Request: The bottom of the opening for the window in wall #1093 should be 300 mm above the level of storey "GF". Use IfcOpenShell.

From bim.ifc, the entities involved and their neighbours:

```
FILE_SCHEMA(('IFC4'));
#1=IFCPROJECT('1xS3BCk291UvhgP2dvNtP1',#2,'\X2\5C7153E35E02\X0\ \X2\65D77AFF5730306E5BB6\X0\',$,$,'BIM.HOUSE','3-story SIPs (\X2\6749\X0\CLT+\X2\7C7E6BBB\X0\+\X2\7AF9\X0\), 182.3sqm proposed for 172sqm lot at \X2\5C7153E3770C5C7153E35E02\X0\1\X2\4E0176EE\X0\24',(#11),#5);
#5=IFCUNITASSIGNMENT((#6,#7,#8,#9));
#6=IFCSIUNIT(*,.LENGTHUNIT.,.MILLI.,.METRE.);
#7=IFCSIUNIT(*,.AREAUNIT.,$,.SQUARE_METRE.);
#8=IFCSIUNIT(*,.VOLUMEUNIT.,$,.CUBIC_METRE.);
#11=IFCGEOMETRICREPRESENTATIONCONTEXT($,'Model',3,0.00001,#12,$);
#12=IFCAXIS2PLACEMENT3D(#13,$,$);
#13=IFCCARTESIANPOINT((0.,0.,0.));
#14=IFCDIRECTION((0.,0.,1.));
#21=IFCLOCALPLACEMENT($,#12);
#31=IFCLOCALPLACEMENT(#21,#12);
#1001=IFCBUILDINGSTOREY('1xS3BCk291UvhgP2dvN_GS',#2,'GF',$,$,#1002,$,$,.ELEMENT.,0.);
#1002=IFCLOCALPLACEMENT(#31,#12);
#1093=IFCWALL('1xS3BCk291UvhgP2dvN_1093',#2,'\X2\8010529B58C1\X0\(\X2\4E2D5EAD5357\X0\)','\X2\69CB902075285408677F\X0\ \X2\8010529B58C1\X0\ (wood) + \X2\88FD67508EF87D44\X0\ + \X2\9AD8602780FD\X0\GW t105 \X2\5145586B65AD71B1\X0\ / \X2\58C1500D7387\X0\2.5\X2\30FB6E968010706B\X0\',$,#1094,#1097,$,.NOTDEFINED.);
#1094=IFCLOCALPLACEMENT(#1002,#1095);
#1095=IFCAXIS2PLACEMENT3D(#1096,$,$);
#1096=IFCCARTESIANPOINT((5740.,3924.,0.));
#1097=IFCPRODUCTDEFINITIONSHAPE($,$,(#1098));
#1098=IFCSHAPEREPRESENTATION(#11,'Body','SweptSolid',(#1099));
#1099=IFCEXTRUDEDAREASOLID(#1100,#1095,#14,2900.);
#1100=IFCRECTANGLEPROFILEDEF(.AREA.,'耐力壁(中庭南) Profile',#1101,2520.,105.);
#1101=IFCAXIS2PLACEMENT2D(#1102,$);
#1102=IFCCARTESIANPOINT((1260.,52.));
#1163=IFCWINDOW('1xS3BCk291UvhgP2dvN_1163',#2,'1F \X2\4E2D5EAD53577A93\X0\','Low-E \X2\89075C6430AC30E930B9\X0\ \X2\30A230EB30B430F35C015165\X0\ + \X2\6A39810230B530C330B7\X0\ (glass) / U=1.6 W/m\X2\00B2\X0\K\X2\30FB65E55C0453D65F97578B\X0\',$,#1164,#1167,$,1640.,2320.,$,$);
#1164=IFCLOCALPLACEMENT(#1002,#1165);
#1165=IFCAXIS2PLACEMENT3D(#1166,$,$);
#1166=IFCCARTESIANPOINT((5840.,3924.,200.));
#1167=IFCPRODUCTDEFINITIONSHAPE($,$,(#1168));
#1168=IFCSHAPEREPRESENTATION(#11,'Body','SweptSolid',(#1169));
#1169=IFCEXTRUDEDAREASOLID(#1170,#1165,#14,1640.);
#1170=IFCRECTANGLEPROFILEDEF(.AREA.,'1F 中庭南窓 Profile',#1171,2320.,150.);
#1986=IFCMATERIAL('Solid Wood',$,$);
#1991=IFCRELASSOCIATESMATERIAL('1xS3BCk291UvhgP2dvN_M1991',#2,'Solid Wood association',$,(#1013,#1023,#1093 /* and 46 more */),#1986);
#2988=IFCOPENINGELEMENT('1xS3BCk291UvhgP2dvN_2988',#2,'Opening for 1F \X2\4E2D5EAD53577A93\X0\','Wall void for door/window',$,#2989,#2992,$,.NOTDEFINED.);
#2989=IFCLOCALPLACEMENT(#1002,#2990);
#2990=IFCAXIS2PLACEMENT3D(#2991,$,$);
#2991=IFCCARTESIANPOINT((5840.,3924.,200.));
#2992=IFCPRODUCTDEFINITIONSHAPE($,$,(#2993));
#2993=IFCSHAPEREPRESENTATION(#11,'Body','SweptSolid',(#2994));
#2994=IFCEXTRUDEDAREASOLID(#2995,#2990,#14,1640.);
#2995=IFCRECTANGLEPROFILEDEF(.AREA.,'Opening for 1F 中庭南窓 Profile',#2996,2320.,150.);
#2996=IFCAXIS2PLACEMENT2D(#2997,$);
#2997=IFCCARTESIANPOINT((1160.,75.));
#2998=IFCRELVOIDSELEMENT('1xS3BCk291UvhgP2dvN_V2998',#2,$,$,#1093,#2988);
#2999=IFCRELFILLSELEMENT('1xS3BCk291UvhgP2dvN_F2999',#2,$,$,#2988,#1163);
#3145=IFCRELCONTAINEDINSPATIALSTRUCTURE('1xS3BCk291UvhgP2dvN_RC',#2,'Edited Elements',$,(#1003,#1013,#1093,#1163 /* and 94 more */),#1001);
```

```python
import numpy as np
import ifcopenshell
import ifcopenshell.api.geometry
import ifcopenshell.geom
import ifcopenshell.util.element
import ifcopenshell.util.placement
import ifcopenshell.util.shape
import ifcopenshell.util.unit

model = ifcopenshell.open("bim.ifc")
unit_scale = ifcopenshell.util.unit.calculate_unit_scale(model)

window = model.by_id(1163)
opening = window.FillsVoids[0].RelatingOpeningElement
storey = ifcopenshell.util.element.get_container(window, ifc_class="IfcBuildingStorey")
level = ifcopenshell.util.placement.get_local_placement(storey.ObjectPlacement)[2, 3]

# The opening's origin need not be at the sill, so measure its lowest point.
shape = ifcopenshell.geom.create_shape(ifcopenshell.geom.settings(), opening)
bottom = ifcopenshell.util.shape.get_shape_bottom_elevation(shape, shape.geometry) / unit_scale
dz = level + 0.3 / unit_scale - bottom

shift = np.array([0.0, 0.0, dz])
# The window is not placed relative to its opening, so move both.
for product in (opening, window):
    matrix = ifcopenshell.util.placement.get_local_placement(product.ObjectPlacement)
    matrix[:3, 3] += shift
    ifcopenshell.api.geometry.edit_object_placement(model, product=product, matrix=matrix, is_si=False)

print(f"moved by {dz * unit_scale:+.3f} m")

model.write("bim_updated.ifc")
```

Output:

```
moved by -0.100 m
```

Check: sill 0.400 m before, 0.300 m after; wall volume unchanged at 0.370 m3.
